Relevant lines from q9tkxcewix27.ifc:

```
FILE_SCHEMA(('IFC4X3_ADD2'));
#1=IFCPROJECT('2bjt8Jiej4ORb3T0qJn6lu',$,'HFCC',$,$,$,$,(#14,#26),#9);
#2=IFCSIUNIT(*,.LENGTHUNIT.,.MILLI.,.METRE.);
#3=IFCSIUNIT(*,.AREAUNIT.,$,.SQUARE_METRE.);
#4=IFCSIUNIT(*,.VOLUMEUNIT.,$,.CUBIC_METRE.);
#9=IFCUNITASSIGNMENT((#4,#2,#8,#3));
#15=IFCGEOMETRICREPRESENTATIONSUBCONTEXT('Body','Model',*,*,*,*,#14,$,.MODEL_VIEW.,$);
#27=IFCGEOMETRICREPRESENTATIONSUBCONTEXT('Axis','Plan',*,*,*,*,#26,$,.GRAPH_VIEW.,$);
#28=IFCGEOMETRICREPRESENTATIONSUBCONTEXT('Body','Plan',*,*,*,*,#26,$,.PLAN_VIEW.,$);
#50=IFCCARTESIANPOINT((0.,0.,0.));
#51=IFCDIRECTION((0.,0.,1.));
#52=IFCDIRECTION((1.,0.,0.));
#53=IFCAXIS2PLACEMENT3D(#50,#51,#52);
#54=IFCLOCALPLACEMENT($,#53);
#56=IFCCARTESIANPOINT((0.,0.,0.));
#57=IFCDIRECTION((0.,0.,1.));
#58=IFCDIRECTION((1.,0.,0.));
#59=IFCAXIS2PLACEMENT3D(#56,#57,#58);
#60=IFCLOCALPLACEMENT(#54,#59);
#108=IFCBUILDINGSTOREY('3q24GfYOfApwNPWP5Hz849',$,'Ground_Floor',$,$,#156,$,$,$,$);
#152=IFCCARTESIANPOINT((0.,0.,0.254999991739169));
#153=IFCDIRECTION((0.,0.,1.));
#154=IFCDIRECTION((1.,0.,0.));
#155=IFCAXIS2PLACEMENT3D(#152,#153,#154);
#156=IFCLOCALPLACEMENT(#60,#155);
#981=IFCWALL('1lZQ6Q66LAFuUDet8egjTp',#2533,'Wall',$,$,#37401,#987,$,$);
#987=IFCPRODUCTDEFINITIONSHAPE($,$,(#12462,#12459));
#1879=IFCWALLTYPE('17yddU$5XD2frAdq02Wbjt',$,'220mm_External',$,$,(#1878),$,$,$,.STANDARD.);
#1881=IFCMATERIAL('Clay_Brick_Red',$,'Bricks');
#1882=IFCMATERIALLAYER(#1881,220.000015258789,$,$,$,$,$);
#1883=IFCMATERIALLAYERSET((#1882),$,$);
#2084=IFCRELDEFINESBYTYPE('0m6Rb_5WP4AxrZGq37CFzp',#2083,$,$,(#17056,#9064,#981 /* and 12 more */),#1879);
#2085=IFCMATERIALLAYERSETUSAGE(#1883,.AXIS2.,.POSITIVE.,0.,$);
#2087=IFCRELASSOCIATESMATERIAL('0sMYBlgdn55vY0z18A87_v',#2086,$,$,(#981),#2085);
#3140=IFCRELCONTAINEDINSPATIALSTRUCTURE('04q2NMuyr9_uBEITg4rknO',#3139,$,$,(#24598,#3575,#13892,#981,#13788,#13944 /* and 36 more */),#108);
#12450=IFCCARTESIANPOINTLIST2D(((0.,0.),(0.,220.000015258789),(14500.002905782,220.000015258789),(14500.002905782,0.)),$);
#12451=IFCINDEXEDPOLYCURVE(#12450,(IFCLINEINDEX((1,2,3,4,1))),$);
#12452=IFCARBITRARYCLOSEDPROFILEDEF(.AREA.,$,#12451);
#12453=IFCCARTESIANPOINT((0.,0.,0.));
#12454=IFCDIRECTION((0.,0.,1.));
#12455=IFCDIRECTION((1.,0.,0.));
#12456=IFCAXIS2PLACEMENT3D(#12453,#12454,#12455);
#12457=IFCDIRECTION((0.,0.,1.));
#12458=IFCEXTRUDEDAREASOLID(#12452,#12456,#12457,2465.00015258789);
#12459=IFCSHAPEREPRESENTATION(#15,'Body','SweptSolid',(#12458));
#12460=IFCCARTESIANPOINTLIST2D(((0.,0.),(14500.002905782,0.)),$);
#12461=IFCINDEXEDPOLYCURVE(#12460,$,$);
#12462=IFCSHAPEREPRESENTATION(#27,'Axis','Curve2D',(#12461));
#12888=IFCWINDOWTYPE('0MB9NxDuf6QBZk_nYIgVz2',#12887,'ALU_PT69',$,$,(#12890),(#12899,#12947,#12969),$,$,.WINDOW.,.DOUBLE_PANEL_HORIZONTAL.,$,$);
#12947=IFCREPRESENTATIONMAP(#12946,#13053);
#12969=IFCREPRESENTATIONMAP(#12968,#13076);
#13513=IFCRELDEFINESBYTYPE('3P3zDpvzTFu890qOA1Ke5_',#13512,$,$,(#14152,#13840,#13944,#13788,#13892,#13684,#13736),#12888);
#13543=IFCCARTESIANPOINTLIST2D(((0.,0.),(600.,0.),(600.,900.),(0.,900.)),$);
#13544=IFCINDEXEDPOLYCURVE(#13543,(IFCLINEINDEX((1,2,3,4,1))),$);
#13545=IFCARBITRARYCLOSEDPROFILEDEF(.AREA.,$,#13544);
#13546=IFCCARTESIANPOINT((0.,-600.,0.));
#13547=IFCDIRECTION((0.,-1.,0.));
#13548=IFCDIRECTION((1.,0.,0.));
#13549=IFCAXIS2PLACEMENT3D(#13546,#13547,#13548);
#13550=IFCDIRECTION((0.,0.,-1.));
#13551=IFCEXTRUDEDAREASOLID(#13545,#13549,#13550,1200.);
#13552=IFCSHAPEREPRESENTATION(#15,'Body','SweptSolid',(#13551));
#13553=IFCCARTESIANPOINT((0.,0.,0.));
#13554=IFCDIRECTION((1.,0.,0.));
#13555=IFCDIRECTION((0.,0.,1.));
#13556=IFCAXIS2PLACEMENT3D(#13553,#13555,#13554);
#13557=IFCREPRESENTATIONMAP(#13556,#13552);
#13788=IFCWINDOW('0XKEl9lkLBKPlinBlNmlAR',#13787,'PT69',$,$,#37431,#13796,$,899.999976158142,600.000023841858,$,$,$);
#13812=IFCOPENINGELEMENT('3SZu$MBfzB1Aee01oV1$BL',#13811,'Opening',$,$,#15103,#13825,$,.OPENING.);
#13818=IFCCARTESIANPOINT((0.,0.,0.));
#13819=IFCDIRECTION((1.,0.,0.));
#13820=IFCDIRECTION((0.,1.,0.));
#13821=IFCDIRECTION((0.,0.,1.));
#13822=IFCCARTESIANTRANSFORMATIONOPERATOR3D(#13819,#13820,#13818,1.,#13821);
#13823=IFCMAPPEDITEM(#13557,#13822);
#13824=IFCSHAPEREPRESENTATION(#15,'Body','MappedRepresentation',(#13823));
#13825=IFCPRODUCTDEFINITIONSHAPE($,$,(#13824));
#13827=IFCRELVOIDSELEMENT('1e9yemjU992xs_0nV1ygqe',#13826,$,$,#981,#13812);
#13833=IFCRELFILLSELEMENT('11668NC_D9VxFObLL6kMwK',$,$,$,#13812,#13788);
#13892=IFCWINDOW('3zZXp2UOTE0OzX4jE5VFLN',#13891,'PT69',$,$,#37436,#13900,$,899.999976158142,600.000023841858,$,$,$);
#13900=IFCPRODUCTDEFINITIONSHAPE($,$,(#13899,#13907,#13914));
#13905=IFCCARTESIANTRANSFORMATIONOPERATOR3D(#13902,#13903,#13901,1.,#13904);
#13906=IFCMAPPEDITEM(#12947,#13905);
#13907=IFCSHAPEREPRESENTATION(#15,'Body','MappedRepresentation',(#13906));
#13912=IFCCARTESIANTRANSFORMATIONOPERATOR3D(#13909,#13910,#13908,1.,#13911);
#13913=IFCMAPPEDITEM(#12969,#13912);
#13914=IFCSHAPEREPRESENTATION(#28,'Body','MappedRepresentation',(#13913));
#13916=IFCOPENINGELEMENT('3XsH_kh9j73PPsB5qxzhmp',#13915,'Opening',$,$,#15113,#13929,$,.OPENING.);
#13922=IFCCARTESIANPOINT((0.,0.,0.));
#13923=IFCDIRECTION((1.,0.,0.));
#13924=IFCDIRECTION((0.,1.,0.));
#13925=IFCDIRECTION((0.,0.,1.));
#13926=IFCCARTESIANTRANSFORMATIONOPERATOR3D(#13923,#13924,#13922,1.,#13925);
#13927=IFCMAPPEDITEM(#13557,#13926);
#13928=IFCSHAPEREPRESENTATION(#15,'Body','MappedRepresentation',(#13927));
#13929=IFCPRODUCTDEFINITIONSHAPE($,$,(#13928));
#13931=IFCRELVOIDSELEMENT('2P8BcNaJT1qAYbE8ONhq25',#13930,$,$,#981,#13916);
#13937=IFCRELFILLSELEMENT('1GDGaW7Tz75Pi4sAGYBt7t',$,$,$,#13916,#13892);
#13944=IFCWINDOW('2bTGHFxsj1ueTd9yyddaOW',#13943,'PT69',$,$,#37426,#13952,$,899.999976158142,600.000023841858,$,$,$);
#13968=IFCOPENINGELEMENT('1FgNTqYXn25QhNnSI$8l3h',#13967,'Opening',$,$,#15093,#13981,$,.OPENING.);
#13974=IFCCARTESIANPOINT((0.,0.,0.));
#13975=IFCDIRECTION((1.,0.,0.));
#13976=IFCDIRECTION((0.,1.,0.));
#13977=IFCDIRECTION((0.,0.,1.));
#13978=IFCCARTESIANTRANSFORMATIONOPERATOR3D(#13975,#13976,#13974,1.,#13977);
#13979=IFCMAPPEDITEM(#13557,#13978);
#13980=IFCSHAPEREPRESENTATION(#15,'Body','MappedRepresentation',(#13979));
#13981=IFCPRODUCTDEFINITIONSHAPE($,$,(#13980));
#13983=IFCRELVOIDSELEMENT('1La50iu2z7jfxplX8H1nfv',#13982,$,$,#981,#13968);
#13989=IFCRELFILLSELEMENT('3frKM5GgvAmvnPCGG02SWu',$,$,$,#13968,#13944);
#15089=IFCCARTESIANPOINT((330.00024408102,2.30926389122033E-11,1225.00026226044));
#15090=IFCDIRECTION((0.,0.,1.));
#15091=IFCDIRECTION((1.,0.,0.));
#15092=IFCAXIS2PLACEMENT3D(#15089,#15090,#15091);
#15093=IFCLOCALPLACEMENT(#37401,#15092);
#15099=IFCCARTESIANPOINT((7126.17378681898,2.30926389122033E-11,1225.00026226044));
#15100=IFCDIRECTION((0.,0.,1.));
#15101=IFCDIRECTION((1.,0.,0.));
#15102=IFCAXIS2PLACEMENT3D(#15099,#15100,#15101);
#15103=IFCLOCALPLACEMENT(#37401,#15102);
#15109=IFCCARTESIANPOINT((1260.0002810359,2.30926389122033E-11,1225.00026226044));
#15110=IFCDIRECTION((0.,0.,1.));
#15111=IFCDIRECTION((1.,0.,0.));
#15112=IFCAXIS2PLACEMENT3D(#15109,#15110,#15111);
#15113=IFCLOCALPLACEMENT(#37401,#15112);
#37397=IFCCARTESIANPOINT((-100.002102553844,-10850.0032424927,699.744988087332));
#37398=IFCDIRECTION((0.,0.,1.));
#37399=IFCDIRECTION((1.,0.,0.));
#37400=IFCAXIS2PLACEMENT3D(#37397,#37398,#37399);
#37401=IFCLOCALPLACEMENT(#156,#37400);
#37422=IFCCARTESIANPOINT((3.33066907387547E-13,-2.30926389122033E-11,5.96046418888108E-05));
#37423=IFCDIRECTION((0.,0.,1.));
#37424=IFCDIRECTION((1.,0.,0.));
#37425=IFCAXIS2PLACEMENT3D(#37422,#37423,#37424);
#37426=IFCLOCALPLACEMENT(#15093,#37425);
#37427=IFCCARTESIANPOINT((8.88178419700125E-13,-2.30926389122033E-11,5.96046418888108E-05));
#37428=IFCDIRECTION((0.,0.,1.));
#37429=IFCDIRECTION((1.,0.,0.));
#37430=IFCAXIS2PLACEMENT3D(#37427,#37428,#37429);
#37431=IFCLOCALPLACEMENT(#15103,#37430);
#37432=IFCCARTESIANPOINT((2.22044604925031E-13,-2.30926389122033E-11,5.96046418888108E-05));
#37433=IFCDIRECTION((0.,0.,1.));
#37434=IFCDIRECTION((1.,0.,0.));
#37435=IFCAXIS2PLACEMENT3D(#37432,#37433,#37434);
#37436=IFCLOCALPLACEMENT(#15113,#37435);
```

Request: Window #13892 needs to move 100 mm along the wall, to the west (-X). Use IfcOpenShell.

```python
import ifcopenshell
import ifcopenshell.api.geometry
import ifcopenshell.util.placement

model = ifcopenshell.open("q9tkxcewix27.ifc")

window = model.by_guid("3zZXp2UOTE0OzX4jE5VFLN")
opening = window.FillsVoids[0].RelatingOpeningElement
wall = opening.VoidsElements[0].RelatingBuildingElement

wall_matrix = ifcopenshell.util.placement.get_local_placement(wall.ObjectPlacement)
shift = wall_matrix[:3, 0] * -100.0
before = ifcopenshell.util.placement.get_local_placement(window.ObjectPlacement)[:3, 3].copy()

# The window is placed relative to its opening, so it follows when the opening moves.
matrix = ifcopenshell.util.placement.get_local_placement(opening.ObjectPlacement)
matrix[:3, 3] += shift
ifcopenshell.api.geometry.edit_object_placement(
    model, product=opening, matrix=matrix, is_si=False, should_transform_children=True
)

after = ifcopenshell.util.placement.get_local_placement(window.ObjectPlacement)[:3, 3]
print("window moved by", (after - before).round(3) + 0.0)

model.write("q9tkxcewix27-out.ifc")
```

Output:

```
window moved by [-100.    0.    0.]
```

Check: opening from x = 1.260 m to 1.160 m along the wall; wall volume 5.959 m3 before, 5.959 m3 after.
